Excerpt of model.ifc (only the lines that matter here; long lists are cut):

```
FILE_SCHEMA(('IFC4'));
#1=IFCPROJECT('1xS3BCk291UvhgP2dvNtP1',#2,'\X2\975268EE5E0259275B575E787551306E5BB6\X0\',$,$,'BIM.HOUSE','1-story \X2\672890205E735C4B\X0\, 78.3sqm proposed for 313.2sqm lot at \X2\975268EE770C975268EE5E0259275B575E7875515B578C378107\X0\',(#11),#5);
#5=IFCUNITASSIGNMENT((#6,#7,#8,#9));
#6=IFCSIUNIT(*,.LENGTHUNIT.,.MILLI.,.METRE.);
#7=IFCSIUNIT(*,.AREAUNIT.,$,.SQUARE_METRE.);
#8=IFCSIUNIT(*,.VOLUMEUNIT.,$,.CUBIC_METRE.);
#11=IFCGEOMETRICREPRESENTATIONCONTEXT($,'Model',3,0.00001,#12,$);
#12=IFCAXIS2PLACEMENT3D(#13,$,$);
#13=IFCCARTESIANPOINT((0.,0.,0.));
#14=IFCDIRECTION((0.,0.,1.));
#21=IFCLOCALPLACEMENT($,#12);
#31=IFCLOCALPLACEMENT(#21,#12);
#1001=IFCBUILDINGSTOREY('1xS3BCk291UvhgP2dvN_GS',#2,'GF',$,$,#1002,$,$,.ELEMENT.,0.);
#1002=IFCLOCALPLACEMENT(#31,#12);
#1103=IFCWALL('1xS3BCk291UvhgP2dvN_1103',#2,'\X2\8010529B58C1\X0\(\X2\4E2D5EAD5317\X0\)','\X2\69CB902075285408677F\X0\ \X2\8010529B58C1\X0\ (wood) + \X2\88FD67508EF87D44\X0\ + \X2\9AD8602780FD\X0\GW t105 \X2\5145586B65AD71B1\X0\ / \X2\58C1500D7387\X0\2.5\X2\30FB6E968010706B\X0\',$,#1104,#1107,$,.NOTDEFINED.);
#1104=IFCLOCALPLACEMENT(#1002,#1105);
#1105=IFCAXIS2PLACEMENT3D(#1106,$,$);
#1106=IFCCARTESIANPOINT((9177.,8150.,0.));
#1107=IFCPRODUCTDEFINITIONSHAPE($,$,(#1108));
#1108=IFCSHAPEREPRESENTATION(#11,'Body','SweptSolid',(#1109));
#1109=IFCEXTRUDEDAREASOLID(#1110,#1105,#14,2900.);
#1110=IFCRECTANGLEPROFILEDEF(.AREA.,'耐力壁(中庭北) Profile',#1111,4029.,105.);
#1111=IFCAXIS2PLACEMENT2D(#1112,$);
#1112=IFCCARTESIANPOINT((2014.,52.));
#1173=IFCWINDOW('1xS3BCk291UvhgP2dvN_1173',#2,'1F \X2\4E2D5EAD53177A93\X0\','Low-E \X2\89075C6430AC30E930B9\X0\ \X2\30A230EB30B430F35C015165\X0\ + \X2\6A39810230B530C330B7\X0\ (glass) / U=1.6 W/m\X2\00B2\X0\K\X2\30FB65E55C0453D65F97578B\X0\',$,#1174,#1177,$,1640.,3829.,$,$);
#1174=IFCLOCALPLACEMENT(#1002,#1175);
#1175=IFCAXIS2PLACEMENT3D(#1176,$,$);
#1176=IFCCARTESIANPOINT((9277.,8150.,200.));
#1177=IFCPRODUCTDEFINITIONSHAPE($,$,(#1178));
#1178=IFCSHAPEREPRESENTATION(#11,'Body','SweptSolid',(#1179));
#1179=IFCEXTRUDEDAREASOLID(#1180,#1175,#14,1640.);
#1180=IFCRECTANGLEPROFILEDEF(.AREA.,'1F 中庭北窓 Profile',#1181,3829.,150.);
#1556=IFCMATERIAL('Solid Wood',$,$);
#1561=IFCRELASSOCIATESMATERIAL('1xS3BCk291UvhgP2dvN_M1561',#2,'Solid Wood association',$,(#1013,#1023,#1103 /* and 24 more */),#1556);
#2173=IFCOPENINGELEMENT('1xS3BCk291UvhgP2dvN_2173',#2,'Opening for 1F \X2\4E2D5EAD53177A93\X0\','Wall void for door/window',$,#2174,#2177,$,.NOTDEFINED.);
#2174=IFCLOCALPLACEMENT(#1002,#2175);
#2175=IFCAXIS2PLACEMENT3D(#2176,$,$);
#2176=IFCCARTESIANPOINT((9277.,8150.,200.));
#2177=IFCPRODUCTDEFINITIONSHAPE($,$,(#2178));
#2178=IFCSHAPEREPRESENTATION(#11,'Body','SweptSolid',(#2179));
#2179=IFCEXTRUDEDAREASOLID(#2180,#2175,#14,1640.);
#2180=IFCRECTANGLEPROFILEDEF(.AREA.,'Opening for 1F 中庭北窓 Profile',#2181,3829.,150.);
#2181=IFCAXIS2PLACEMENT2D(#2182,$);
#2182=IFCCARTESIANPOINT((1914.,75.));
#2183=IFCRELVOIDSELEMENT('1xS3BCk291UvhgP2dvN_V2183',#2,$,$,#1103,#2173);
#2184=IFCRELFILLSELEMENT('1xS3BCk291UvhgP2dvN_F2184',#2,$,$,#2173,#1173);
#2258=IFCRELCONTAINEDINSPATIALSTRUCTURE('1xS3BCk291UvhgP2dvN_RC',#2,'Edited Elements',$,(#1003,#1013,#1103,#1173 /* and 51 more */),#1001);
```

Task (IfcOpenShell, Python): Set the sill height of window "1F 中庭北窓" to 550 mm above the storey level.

```python
import numpy as np
import ifcopenshell
import ifcopenshell.api.geometry
import ifcopenshell.geom
import ifcopenshell.util.element
import ifcopenshell.util.placement
import ifcopenshell.util.shape
import ifcopenshell.util.unit

model = ifcopenshell.open("model.ifc")
unit_scale = ifcopenshell.util.unit.calculate_unit_scale(model)

window = model.by_guid("1xS3BCk291UvhgP2dvN_1173")
opening = window.FillsVoids[0].RelatingOpeningElement
storey = ifcopenshell.util.element.get_container(window, ifc_class="IfcBuildingStorey")
level = ifcopenshell.util.placement.get_local_placement(storey.ObjectPlacement)[2, 3]

# The opening's origin need not be at the sill, so measure its lowest point.
shape = ifcopenshell.geom.create_shape(ifcopenshell.geom.settings(), opening)
bottom = ifcopenshell.util.shape.get_shape_bottom_elevation(shape, shape.geometry) / unit_scale
dz = level + 0.55 / unit_scale - bottom

shift = np.array([0.0, 0.0, dz])
# The window is not placed relative to its opening, so move both.
for product in (opening, window):
    matrix = ifcopenshell.util.placement.get_local_placement(product.ObjectPlacement)
    matrix[:3, 3] += shift
    ifcopenshell.api.geometry.edit_object_placement(model, product=product, matrix=matrix, is_si=False)

print(f"moved by {dz * unit_scale:+.3f} m")

model.write("model_rev.ifc")
```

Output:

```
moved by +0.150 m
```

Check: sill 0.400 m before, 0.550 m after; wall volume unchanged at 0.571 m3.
